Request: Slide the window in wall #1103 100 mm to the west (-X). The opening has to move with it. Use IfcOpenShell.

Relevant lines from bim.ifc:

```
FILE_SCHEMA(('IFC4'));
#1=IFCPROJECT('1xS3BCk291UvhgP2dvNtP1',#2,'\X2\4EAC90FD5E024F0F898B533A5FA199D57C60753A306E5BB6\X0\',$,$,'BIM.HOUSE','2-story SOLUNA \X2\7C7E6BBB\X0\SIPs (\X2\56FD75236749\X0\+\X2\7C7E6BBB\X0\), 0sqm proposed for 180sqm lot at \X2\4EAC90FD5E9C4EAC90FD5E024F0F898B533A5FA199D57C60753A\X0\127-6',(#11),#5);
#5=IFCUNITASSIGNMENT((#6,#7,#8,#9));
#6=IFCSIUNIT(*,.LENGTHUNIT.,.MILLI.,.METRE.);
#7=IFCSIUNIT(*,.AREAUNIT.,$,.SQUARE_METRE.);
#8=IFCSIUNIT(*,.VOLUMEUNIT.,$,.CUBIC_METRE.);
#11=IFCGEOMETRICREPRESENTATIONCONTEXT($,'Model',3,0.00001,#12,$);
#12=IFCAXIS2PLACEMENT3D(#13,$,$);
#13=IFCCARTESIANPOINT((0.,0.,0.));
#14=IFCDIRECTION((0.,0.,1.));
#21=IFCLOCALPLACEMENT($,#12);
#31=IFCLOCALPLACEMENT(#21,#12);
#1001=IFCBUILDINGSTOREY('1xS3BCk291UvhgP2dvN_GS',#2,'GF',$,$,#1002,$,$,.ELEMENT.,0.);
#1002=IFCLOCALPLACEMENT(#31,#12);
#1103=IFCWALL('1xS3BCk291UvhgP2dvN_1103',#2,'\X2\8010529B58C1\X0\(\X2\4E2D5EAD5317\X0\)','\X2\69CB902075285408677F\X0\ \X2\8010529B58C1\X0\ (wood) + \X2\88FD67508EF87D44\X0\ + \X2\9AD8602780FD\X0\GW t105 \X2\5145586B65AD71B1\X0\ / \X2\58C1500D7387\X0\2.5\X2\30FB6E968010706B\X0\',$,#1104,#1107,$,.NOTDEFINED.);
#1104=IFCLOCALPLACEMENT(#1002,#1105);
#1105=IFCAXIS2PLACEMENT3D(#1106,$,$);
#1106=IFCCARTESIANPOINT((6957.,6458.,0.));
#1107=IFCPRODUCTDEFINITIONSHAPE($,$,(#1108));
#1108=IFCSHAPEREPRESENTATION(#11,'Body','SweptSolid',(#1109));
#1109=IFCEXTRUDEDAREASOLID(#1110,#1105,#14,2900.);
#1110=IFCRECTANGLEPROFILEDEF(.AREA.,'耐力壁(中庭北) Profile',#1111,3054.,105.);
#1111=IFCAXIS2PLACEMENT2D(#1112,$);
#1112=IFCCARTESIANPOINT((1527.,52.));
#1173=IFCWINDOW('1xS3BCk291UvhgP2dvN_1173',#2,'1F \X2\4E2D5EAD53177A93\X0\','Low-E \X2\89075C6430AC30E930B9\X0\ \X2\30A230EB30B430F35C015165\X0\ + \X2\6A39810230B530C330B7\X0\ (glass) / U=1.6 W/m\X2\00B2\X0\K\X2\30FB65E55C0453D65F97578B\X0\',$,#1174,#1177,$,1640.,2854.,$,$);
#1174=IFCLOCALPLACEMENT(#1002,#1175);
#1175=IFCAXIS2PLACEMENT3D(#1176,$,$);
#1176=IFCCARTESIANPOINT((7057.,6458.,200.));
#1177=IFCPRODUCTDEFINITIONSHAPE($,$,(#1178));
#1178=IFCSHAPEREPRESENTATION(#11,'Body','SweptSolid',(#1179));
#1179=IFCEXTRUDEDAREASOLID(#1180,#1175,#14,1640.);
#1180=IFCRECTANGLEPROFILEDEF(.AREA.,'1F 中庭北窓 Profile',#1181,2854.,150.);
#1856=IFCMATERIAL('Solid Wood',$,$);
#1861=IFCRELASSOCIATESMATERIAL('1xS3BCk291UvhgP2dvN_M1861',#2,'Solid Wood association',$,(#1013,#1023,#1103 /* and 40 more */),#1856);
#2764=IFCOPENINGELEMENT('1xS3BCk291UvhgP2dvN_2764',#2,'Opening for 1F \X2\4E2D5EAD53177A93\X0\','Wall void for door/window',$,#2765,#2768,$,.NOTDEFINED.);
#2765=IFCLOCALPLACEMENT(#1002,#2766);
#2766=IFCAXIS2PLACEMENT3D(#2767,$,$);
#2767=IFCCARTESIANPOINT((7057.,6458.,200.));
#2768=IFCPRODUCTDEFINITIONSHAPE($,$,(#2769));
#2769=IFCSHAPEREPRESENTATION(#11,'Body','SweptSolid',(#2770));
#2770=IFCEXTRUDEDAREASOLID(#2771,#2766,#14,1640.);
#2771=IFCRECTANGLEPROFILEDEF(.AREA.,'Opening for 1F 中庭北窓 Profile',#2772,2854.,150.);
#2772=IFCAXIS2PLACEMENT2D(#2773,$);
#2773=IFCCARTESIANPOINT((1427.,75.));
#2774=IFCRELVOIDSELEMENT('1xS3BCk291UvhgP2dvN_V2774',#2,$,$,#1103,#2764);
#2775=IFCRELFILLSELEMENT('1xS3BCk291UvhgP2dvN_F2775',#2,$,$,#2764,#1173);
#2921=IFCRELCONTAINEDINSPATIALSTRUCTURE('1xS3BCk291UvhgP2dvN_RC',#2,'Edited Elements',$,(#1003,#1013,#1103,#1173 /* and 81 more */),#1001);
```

```python
import ifcopenshell
import ifcopenshell.api.geometry
import ifcopenshell.util.placement

model = ifcopenshell.open("bim.ifc")

window = model.by_guid("1xS3BCk291UvhgP2dvN_1173")
opening = window.FillsVoids[0].RelatingOpeningElement
wall = opening.VoidsElements[0].RelatingBuildingElement

wall_matrix = ifcopenshell.util.placement.get_local_placement(wall.ObjectPlacement)
shift = wall_matrix[:3, 0] * -100.0
before = ifcopenshell.util.placement.get_local_placement(window.ObjectPlacement)[:3, 3].copy()

# The window is not placed relative to its opening, so move both.
for product in (opening, window):
    matrix = ifcopenshell.util.placement.get_local_placement(product.ObjectPlacement)
    matrix[:3, 3] += shift
    ifcopenshell.api.geometry.edit_object_placement(model, product=product, matrix=matrix, is_si=False)

after = ifcopenshell.util.placement.get_local_placement(window.ObjectPlacement)[:3, 3]
print("window moved by", (after - before).round(3) + 0.0)

model.write("bim-out.ifc")
```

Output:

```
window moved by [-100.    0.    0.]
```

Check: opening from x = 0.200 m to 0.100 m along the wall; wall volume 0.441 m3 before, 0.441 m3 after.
